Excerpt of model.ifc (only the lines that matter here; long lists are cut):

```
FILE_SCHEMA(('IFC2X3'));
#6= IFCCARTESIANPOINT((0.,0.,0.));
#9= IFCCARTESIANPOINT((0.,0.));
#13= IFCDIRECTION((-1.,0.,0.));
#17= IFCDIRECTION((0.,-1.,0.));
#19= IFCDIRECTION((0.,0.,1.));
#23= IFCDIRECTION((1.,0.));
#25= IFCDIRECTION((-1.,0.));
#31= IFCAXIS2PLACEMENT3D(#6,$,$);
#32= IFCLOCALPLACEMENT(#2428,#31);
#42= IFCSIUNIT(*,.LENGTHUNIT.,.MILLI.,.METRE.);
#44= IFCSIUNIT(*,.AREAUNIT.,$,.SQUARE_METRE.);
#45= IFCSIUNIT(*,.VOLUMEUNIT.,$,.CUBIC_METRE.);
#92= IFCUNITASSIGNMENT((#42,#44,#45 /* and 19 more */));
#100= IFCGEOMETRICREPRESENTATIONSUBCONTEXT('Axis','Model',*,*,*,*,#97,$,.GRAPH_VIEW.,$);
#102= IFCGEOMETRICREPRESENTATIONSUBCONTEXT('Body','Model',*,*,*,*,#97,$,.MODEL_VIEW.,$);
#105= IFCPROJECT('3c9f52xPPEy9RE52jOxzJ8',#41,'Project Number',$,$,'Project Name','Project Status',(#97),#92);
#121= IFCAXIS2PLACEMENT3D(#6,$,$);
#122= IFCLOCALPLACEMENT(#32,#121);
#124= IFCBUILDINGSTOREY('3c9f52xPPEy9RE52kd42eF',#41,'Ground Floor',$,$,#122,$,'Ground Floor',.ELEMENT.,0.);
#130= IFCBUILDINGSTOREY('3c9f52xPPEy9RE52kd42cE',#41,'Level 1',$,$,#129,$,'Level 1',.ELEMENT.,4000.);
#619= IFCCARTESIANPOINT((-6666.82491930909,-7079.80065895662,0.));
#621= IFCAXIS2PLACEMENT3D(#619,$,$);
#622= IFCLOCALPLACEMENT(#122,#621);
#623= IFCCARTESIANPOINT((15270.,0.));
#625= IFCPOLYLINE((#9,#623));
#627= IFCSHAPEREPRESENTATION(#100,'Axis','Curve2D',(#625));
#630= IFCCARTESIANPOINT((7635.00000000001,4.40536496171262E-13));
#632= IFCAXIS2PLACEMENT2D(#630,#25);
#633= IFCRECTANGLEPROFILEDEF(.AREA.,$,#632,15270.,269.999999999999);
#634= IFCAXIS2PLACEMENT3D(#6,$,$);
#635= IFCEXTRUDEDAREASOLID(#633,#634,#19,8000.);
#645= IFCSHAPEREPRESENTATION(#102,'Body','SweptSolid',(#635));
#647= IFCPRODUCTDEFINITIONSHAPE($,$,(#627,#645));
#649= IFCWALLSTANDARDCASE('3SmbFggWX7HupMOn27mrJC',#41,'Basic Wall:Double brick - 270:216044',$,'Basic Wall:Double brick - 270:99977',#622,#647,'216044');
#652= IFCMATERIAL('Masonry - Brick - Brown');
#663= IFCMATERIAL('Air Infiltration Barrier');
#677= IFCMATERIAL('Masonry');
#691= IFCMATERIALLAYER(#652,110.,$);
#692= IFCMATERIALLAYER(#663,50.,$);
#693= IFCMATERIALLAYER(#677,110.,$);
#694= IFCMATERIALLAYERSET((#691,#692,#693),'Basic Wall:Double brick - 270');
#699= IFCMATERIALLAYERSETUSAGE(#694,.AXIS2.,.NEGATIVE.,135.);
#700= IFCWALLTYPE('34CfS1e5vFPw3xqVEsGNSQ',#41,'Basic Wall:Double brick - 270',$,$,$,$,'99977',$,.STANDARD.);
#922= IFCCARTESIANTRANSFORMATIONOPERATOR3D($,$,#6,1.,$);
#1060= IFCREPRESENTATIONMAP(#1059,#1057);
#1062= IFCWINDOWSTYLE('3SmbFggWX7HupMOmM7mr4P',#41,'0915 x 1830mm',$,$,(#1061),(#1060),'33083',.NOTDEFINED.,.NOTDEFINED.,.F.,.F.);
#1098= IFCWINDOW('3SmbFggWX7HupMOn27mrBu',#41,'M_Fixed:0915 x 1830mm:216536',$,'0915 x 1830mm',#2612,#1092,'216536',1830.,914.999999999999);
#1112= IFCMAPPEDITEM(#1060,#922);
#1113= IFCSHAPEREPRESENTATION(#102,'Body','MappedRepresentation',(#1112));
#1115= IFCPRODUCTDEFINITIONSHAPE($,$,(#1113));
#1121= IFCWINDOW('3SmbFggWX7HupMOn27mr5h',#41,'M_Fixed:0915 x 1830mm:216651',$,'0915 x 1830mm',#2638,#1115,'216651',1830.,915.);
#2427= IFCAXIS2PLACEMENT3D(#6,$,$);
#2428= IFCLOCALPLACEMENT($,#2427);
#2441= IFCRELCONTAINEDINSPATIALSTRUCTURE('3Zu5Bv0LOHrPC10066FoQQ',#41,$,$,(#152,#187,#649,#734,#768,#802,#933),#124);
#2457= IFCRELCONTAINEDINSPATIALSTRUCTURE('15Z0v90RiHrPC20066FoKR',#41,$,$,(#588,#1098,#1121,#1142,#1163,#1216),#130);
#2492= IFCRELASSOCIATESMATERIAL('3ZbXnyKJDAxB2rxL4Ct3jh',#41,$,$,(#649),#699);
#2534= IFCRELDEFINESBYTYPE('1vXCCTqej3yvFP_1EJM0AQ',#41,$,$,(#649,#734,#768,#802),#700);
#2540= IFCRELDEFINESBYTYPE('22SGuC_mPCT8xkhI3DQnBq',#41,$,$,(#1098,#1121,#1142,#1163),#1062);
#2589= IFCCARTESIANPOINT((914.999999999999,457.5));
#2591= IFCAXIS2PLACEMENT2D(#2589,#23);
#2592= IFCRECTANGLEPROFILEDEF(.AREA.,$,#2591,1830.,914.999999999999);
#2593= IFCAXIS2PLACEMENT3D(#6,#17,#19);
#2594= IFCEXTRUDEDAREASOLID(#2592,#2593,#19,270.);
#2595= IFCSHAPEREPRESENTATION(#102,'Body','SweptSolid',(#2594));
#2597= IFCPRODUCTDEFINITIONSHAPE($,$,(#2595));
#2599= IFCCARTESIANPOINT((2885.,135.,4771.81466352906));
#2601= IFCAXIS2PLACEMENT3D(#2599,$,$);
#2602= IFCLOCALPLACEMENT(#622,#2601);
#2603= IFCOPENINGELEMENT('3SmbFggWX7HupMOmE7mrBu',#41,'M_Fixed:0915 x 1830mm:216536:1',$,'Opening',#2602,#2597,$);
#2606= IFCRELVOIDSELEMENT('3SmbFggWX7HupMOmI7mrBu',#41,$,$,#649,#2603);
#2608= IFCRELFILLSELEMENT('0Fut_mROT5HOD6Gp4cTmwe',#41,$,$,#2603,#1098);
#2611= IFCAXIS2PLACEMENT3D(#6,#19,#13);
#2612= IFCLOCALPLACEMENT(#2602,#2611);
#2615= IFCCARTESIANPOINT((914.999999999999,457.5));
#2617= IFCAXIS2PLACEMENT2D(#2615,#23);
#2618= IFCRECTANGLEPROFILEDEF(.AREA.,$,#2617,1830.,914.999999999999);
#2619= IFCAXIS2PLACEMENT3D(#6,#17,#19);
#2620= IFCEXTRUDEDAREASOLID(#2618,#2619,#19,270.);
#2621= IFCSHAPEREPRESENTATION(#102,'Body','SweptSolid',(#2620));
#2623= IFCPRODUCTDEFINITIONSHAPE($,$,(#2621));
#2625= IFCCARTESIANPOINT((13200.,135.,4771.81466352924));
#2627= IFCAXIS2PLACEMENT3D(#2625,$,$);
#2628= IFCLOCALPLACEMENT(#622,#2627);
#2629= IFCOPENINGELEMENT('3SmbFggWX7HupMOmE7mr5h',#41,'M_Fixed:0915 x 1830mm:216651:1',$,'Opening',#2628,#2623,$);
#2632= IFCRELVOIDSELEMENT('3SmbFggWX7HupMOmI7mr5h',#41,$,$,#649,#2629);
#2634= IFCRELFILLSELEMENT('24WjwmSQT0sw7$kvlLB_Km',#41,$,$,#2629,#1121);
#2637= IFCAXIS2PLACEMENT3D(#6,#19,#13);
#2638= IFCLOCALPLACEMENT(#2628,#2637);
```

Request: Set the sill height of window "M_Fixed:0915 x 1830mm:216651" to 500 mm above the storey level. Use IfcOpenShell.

```python
import numpy as np
import ifcopenshell
import ifcopenshell.api.geometry
import ifcopenshell.geom
import ifcopenshell.util.element
import ifcopenshell.util.placement
import ifcopenshell.util.shape
import ifcopenshell.util.unit

model = ifcopenshell.open("model.ifc")
unit_scale = ifcopenshell.util.unit.calculate_unit_scale(model)

window = model.by_guid("3SmbFggWX7HupMOn27mr5h")
opening = window.FillsVoids[0].RelatingOpeningElement
storey = ifcopenshell.util.element.get_container(window, ifc_class="IfcBuildingStorey")
level = ifcopenshell.util.placement.get_local_placement(storey.ObjectPlacement)[2, 3]

# The opening's origin need not be at the sill, so measure its lowest point.
shape = ifcopenshell.geom.create_shape(ifcopenshell.geom.settings(), opening)
bottom = ifcopenshell.util.shape.get_shape_bottom_elevation(shape, shape.geometry) / unit_scale
dz = level + 500.0 - bottom

shift = np.array([0.0, 0.0, dz])
# The window is placed relative to its opening, so it follows when the opening moves.
matrix = ifcopenshell.util.placement.get_local_placement(opening.ObjectPlacement)
matrix[:3, 3] += shift
ifcopenshell.api.geometry.edit_object_placement(
    model, product=opening, matrix=matrix, is_si=False, should_transform_children=True
)

print(f"moved by {dz * unit_scale:+.3f} m")

model.write("model_rev.ifc")
```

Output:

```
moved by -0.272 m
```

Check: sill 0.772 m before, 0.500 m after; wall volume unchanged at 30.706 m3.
